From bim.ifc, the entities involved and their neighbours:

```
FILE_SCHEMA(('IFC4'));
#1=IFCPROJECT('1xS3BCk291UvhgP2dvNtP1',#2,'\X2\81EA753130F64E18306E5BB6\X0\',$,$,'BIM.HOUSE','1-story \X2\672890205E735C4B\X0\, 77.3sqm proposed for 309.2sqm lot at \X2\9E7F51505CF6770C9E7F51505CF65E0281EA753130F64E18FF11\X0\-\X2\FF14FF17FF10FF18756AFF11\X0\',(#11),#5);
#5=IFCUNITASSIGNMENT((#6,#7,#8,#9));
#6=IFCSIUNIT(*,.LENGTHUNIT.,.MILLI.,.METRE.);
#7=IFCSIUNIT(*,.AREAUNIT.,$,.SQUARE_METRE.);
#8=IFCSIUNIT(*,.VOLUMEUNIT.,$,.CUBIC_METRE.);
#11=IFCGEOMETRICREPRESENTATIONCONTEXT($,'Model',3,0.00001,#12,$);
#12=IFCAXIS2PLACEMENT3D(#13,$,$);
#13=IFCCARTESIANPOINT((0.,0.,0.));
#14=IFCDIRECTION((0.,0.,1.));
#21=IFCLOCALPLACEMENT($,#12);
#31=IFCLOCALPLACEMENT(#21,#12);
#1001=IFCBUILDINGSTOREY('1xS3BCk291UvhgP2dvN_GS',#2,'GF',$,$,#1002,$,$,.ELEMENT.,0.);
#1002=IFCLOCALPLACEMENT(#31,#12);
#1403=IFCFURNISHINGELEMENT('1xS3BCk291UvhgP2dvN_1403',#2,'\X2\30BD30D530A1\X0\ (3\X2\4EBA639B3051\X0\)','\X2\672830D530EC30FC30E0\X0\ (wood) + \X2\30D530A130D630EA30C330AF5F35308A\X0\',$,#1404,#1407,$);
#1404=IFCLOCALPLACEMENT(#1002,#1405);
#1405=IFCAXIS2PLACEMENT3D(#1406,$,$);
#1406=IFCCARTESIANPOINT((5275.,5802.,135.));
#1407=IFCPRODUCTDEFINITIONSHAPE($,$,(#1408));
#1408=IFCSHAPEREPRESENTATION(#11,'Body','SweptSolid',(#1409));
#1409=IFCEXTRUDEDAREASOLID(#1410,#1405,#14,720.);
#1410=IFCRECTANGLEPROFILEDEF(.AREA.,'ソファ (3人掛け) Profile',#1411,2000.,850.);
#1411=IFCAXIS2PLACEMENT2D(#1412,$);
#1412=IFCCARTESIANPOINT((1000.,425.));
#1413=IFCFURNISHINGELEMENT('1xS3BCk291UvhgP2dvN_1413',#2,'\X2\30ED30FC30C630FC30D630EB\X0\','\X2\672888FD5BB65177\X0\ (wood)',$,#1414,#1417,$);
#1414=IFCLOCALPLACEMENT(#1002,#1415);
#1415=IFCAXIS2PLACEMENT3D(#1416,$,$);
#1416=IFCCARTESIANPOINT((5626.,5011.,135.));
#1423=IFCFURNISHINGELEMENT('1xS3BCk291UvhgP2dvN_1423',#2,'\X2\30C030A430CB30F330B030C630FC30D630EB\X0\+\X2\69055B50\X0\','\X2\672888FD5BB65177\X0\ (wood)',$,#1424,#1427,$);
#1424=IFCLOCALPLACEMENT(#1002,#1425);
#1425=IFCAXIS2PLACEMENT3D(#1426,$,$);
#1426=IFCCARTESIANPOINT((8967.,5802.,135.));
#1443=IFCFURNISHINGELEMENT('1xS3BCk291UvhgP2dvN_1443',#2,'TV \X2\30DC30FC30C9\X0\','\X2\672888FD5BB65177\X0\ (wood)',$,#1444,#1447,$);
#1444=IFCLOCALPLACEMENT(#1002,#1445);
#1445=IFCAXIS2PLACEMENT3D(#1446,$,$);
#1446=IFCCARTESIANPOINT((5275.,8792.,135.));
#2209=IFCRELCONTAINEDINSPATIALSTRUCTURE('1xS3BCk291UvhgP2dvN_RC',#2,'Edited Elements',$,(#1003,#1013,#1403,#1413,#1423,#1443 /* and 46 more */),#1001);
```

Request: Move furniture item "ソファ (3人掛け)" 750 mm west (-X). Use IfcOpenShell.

```python
import ifcopenshell
import ifcopenshell.api.geometry
import ifcopenshell.util.placement
import ifcopenshell.util.unit

model = ifcopenshell.open("bim.ifc")
unit_scale = ifcopenshell.util.unit.calculate_unit_scale(model)

item = model.by_guid("1xS3BCk291UvhgP2dvN_1403")
matrix = ifcopenshell.util.placement.get_local_placement(item.ObjectPlacement)
matrix[0, 3] -= 0.75 / unit_scale
ifcopenshell.api.geometry.edit_object_placement(model, product=item, matrix=matrix, is_si=False)

print(ifcopenshell.util.placement.get_local_placement(item.ObjectPlacement).round(3) + 0.0)

model.write("bim_updated.ifc")
```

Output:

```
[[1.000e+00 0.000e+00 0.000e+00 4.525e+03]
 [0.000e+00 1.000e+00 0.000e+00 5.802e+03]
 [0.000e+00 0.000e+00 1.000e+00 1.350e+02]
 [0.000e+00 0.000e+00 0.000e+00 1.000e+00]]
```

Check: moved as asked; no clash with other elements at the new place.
